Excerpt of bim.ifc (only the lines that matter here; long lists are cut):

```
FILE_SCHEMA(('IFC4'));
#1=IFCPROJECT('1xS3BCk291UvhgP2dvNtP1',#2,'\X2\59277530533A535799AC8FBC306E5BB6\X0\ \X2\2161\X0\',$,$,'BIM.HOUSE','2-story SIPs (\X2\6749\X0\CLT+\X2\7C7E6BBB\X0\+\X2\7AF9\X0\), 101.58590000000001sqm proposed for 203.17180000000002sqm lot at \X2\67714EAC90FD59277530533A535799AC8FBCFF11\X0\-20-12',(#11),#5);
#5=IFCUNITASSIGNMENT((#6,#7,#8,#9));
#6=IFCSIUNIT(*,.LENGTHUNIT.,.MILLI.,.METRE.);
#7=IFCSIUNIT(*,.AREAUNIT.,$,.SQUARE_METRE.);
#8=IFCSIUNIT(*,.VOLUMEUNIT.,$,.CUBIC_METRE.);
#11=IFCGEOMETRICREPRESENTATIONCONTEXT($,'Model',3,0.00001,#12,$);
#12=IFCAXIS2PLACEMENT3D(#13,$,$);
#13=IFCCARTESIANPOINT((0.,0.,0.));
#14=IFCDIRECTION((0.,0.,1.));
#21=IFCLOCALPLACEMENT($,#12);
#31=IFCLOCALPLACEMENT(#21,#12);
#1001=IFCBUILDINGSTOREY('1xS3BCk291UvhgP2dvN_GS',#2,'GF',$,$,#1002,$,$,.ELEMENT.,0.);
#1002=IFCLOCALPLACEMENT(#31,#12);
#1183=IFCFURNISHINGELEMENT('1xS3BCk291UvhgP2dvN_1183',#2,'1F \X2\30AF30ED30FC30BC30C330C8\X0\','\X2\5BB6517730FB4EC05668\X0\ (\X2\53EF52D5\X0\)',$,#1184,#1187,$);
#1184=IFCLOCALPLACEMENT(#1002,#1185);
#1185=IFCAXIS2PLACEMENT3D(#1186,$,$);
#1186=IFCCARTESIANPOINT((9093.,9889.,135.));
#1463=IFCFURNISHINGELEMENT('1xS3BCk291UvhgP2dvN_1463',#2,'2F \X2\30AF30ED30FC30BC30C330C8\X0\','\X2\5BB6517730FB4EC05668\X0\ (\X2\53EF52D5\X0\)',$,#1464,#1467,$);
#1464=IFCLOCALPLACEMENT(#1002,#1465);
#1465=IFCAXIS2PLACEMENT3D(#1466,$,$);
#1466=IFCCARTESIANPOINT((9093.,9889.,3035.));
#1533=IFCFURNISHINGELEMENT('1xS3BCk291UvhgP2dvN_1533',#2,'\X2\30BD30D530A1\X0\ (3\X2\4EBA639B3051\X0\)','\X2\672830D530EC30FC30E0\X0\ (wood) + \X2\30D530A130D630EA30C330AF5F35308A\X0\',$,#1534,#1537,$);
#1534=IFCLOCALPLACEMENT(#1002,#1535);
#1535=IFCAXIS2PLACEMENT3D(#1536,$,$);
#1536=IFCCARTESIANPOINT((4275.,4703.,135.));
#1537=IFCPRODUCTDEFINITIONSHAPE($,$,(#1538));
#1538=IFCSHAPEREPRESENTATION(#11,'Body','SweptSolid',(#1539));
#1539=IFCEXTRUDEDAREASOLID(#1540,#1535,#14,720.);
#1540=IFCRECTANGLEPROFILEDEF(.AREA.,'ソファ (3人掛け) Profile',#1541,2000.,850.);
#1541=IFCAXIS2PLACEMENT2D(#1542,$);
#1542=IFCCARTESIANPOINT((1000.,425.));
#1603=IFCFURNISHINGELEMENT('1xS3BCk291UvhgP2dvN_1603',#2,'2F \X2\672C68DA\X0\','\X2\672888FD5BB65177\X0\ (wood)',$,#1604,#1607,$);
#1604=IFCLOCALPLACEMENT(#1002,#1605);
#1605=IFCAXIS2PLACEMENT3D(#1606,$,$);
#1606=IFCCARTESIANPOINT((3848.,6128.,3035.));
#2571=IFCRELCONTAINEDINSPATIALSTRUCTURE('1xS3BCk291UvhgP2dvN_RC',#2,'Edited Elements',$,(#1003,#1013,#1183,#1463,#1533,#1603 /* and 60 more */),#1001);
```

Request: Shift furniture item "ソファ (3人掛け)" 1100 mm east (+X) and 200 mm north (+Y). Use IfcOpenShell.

```python
import ifcopenshell
import ifcopenshell.api.geometry
import ifcopenshell.util.placement

model = ifcopenshell.open("bim.ifc")

item = model.by_guid("1xS3BCk291UvhgP2dvN_1533")
matrix = ifcopenshell.util.placement.get_local_placement(item.ObjectPlacement)
matrix[0, 3] += 1100.0
matrix[1, 3] += 200.0
ifcopenshell.api.geometry.edit_object_placement(model, product=item, matrix=matrix, is_si=False)

print(ifcopenshell.util.placement.get_local_placement(item.ObjectPlacement).round(3) + 0.0)

model.write("bim-out.ifc")
```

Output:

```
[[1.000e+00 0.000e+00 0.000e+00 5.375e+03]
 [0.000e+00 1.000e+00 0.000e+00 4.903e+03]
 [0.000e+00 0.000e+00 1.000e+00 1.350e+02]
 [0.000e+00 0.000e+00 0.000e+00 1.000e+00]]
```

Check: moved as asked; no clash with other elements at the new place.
